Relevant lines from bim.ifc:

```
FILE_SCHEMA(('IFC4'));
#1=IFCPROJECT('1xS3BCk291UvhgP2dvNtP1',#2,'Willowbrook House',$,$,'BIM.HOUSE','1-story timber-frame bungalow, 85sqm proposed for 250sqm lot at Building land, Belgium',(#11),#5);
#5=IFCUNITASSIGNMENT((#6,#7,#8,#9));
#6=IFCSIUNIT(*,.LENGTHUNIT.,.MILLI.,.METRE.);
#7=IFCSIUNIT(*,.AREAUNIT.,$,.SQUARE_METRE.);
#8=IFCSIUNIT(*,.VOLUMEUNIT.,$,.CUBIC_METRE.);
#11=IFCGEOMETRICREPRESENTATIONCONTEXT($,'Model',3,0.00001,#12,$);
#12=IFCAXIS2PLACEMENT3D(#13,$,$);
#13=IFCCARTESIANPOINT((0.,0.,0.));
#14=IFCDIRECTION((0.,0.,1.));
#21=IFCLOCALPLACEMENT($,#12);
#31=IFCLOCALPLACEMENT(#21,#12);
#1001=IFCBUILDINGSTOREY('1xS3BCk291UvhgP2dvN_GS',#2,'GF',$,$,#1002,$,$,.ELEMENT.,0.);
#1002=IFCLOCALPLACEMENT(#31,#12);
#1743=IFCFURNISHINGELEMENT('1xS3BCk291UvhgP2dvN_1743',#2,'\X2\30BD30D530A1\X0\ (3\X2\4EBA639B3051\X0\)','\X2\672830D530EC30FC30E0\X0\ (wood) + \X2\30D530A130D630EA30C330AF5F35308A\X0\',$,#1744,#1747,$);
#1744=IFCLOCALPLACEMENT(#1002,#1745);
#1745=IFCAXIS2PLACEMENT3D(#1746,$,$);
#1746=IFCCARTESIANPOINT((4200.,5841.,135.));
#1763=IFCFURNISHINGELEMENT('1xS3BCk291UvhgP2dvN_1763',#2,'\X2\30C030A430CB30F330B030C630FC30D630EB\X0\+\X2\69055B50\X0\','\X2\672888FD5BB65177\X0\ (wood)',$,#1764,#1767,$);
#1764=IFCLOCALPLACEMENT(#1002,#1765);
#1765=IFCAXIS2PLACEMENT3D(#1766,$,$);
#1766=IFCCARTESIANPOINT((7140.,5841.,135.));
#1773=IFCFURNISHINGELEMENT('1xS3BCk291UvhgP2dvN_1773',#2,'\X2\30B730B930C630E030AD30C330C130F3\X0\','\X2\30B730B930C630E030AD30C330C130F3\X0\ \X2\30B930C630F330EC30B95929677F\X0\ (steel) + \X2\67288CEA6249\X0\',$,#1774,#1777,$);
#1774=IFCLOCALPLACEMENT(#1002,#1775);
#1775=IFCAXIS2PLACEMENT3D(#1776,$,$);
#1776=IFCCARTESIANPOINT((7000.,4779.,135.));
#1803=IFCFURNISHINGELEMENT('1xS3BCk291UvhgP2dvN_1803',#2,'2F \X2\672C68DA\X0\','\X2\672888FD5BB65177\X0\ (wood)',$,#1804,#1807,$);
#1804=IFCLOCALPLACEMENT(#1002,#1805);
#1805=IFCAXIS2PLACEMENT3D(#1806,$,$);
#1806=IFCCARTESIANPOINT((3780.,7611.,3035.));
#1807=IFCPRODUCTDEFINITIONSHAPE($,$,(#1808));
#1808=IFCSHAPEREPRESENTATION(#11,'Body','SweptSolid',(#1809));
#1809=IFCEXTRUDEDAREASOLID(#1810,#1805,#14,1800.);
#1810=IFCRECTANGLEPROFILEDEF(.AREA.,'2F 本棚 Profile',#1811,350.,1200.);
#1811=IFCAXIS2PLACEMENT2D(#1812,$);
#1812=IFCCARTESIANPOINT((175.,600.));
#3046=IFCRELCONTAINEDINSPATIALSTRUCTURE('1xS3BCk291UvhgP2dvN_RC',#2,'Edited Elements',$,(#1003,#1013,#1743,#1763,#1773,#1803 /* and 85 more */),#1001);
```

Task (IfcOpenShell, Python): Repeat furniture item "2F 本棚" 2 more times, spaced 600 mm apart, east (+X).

```python
import numpy as np
import ifcopenshell
import ifcopenshell.api.geometry
import ifcopenshell.api.root
import ifcopenshell.util.element
import ifcopenshell.util.placement

model = ifcopenshell.open("bim.ifc")


def reuse_history(source, copy):
    """copy_class also copies each property set's owner history, people and application; keep the originals."""
    for rel in copy.IsDefinedBy:
        if rel.is_a("IfcRelDefinesByProperties") and (history := rel.RelatingPropertyDefinition.OwnerHistory):
            rel.RelatingPropertyDefinition.OwnerHistory = source.OwnerHistory
            ifcopenshell.util.element.remove_deep2(model, history)


source = model.by_guid("1xS3BCk291UvhgP2dvN_1803")
base = ifcopenshell.util.placement.get_local_placement(source.ObjectPlacement)
step = np.array([1.0, 0.0, 0.0]) * 600.0

for i in range(1, 3):
    copy = ifcopenshell.api.root.copy_class(model, product=source)
    copy.Representation = ifcopenshell.util.element.copy_deep(
        model, source.Representation, exclude=["IfcGeometricRepresentationContext", "IfcRepresentationMap"]
    )
    reuse_history(source, copy)
    matrix = base.copy()
    matrix[:3, 3] += i * step
    print("added at", matrix[:3, 3].round(3) + 0.0)
    ifcopenshell.api.geometry.edit_object_placement(model, product=copy, matrix=matrix, is_si=False)

model.write("bim_updated.ifc")
```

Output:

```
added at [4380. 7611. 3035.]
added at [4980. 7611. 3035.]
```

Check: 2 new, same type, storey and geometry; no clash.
